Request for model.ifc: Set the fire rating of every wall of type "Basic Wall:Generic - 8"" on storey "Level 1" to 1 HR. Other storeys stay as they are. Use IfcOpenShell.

First a look at what the model holds.

```python
import ifcopenshell
import ifcopenshell.util.element

model = ifcopenshell.open("model.ifc")
print(model.schema)
storey = next(s for s in model.by_type("IfcBuildingStorey") if s.Name == "Level 1")
walls = [e for e in ifcopenshell.util.element.get_decomposition(storey) if e.is_a("IfcWall")]
seen = {}
for e in walls:
    element_type = ifcopenshell.util.element.get_type(e)
    key = (element_type.Name if element_type != e and element_type else None, ifcopenshell.util.element.get_pset(e, "Pset_WallCommon", "FireRating"))
    seen[key] = seen.get(key, 0) + 1
for (name, value), count in sorted(seen.items(), key=str):
    print(count, "x", name, "|", value)
```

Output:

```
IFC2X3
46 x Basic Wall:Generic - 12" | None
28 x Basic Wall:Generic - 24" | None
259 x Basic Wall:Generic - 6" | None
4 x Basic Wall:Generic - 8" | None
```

```python
import ifcopenshell
import ifcopenshell.api.pset
import ifcopenshell.util.element

model = ifcopenshell.open("model.ifc")

storey = next(s for s in model.by_type("IfcBuildingStorey") if s.Name == "Level 1")
walls = [e for e in ifcopenshell.util.element.get_decomposition(storey) if e.is_a("IfcWall")]

count = 0
for e in walls:
    element_type = ifcopenshell.util.element.get_type(e)
    if element_type in (None, e) or element_type.Name != 'Basic Wall:Generic - 8"':
        continue
    # add_pset returns the element's existing set when there is one.
    pset = ifcopenshell.api.pset.add_pset(model, product=e, name="Pset_WallCommon")
    ifcopenshell.api.pset.edit_pset(model, pset=pset, properties={"FireRating": "1 HR"})
    count += 1

print(count, "walls updated")

model.write("model_v2.ifc")
```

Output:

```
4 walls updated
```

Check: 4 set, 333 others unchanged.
